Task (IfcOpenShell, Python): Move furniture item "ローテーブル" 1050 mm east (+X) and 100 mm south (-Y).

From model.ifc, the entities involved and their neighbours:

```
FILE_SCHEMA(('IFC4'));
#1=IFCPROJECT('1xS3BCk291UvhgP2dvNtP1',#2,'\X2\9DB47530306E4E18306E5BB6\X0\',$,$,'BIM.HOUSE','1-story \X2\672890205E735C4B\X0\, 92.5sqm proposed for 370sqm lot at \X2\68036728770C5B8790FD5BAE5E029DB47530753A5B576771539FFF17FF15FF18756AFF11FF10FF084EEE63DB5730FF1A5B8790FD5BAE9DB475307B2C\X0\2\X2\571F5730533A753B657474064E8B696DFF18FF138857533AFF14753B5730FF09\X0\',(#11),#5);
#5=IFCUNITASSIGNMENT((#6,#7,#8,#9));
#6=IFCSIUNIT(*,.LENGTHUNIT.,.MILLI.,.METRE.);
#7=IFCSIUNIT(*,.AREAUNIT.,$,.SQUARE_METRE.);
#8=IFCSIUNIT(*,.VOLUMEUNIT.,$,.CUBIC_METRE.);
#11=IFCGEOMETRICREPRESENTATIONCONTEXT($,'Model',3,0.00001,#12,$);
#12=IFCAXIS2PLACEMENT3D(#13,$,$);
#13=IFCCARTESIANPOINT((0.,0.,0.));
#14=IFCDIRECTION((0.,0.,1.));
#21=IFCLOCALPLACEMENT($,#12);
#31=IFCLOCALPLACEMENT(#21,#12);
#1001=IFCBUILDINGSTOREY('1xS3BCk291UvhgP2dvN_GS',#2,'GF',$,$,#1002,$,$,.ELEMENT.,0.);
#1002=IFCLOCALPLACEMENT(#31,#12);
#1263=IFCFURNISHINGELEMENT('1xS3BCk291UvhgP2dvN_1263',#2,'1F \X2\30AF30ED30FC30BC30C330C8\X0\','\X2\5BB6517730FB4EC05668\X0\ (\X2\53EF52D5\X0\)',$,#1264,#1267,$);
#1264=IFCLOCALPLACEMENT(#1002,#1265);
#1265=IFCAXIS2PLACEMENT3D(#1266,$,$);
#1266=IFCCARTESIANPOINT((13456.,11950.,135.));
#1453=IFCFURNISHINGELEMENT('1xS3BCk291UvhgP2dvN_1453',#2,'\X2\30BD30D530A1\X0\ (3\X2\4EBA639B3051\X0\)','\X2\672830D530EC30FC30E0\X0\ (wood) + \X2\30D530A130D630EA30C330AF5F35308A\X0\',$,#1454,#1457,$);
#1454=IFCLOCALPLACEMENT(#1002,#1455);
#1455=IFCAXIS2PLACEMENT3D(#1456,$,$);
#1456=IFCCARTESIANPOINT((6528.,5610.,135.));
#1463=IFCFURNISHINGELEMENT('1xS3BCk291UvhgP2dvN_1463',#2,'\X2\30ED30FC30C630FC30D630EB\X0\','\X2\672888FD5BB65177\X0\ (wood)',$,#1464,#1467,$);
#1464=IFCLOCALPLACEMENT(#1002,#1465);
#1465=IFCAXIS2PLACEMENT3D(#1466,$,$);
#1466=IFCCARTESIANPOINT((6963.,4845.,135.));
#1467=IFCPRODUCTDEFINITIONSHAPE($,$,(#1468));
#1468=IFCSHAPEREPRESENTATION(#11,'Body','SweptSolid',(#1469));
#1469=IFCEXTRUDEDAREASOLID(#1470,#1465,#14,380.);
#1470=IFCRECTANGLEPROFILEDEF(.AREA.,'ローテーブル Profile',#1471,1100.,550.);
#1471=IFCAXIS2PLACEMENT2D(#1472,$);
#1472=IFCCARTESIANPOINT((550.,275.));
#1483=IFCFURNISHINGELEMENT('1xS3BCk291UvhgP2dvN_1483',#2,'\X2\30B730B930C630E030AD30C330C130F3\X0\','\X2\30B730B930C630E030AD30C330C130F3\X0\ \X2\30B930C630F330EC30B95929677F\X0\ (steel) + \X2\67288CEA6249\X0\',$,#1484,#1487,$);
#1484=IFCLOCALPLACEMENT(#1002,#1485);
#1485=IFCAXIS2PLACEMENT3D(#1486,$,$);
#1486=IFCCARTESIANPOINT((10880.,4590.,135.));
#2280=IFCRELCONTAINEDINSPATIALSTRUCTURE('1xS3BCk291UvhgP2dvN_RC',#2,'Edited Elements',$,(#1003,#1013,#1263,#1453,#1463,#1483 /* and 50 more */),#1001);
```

```python
import ifcopenshell
import ifcopenshell.api.geometry
import ifcopenshell.util.placement
import ifcopenshell.util.unit

model = ifcopenshell.open("model.ifc")
unit_scale = ifcopenshell.util.unit.calculate_unit_scale(model)

item = model.by_guid("1xS3BCk291UvhgP2dvN_1463")
matrix = ifcopenshell.util.placement.get_local_placement(item.ObjectPlacement)
matrix[0, 3] += 1.05 / unit_scale
matrix[1, 3] -= 0.1 / unit_scale
ifcopenshell.api.geometry.edit_object_placement(model, product=item, matrix=matrix, is_si=False)

print(ifcopenshell.util.placement.get_local_placement(item.ObjectPlacement).round(3) + 0.0)

model.write("model_rev.ifc")
```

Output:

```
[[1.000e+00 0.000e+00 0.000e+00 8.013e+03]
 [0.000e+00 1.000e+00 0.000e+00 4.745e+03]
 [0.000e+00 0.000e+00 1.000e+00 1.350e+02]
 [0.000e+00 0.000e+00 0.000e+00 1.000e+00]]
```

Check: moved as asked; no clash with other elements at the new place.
